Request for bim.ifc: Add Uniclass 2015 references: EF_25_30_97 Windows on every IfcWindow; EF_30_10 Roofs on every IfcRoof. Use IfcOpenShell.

First a look at what the model holds.

```python
import ifcopenshell

model = ifcopenshell.open("bim.ifc")
print(model.schema)
print("classifications:", [c.Name for c in model.by_type("IfcClassification")])
for ifc_class in ("IfcDoor", "IfcRoof", "IfcStair", "IfcWall", "IfcWindow"):
    print(ifc_class, len(model.by_type(ifc_class)))
```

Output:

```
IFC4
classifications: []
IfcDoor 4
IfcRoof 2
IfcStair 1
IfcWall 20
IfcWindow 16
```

```python
import ifcopenshell
import ifcopenshell.api.classification

model = ifcopenshell.open("bim.ifc")

system = ifcopenshell.api.classification.add_classification(model, classification="Uniclass 2015")

codes = {
    "IfcWindow": ("EF_25_30_97", "Windows"),
    "IfcRoof": ("EF_30_10", "Roofs"),
}
for ifc_class, (code, name) in codes.items():
    products = model.by_type(ifc_class)
    ifcopenshell.api.classification.add_reference(
        model, products=products, classification=system, identification=code, name=name
    )
    print(code, len(products))

model.write("bim_rev.ifc")
```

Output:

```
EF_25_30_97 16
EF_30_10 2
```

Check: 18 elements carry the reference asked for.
